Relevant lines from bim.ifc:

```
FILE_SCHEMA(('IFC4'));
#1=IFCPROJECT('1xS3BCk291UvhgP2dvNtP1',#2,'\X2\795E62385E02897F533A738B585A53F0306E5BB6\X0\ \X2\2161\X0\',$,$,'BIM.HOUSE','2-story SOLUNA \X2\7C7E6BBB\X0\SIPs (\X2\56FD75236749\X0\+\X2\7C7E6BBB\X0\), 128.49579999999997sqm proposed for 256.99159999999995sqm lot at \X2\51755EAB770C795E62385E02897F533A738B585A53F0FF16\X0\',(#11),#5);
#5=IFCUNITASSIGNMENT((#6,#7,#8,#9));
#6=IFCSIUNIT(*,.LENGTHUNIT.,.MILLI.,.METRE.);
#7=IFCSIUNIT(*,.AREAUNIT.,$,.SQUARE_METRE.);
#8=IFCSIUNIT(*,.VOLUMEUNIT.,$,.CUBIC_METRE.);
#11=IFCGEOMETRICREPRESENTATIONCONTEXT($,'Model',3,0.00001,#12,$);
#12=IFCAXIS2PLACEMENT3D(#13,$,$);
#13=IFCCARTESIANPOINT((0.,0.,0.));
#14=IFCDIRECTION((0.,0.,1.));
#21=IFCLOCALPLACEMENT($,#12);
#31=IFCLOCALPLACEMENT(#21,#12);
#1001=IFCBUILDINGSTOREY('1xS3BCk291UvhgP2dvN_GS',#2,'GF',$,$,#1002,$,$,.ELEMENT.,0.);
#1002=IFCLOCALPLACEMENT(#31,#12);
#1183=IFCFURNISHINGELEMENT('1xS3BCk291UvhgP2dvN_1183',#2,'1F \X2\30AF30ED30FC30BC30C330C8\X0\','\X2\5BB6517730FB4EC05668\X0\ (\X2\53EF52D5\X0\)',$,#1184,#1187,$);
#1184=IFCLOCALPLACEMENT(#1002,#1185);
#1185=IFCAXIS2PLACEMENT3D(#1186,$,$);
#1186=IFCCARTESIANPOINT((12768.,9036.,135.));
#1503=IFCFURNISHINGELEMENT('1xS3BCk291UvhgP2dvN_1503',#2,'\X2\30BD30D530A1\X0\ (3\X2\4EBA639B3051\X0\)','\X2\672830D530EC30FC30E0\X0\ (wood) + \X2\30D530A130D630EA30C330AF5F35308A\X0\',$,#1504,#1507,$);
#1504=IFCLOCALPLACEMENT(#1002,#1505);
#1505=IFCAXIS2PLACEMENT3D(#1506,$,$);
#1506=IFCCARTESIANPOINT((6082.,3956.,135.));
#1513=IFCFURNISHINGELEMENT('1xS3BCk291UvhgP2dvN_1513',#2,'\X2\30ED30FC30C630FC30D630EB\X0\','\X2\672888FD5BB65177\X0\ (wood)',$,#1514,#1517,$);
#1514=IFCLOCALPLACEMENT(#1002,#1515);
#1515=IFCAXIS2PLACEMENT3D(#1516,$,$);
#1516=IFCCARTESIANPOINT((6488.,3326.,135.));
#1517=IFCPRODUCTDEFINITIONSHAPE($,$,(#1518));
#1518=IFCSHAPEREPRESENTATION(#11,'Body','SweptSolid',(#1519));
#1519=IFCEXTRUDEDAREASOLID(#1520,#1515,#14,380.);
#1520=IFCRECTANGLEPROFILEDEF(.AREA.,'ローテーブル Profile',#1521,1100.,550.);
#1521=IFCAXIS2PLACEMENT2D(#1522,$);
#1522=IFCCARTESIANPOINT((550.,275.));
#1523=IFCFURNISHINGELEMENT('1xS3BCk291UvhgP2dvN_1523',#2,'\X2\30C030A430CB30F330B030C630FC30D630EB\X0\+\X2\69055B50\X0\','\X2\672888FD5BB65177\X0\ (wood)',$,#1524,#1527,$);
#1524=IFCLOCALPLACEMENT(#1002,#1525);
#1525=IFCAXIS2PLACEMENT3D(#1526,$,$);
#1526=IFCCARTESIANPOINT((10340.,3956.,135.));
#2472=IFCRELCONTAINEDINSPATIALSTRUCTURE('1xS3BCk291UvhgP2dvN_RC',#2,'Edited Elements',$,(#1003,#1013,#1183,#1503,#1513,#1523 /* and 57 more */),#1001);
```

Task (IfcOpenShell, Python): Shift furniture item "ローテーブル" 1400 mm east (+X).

```python
import ifcopenshell
import ifcopenshell.api.geometry
import ifcopenshell.util.placement
import ifcopenshell.util.unit

model = ifcopenshell.open("bim.ifc")
unit_scale = ifcopenshell.util.unit.calculate_unit_scale(model)

item = model.by_guid("1xS3BCk291UvhgP2dvN_1513")
matrix = ifcopenshell.util.placement.get_local_placement(item.ObjectPlacement)
matrix[0, 3] += 1.4 / unit_scale
ifcopenshell.api.geometry.edit_object_placement(model, product=item, matrix=matrix, is_si=False)

print(ifcopenshell.util.placement.get_local_placement(item.ObjectPlacement).round(3) + 0.0)

model.write("bim_rev.ifc")
```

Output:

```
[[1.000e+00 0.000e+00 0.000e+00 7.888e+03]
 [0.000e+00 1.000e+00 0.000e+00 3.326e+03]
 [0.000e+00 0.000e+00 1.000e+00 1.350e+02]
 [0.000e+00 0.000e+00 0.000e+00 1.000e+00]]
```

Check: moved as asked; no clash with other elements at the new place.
